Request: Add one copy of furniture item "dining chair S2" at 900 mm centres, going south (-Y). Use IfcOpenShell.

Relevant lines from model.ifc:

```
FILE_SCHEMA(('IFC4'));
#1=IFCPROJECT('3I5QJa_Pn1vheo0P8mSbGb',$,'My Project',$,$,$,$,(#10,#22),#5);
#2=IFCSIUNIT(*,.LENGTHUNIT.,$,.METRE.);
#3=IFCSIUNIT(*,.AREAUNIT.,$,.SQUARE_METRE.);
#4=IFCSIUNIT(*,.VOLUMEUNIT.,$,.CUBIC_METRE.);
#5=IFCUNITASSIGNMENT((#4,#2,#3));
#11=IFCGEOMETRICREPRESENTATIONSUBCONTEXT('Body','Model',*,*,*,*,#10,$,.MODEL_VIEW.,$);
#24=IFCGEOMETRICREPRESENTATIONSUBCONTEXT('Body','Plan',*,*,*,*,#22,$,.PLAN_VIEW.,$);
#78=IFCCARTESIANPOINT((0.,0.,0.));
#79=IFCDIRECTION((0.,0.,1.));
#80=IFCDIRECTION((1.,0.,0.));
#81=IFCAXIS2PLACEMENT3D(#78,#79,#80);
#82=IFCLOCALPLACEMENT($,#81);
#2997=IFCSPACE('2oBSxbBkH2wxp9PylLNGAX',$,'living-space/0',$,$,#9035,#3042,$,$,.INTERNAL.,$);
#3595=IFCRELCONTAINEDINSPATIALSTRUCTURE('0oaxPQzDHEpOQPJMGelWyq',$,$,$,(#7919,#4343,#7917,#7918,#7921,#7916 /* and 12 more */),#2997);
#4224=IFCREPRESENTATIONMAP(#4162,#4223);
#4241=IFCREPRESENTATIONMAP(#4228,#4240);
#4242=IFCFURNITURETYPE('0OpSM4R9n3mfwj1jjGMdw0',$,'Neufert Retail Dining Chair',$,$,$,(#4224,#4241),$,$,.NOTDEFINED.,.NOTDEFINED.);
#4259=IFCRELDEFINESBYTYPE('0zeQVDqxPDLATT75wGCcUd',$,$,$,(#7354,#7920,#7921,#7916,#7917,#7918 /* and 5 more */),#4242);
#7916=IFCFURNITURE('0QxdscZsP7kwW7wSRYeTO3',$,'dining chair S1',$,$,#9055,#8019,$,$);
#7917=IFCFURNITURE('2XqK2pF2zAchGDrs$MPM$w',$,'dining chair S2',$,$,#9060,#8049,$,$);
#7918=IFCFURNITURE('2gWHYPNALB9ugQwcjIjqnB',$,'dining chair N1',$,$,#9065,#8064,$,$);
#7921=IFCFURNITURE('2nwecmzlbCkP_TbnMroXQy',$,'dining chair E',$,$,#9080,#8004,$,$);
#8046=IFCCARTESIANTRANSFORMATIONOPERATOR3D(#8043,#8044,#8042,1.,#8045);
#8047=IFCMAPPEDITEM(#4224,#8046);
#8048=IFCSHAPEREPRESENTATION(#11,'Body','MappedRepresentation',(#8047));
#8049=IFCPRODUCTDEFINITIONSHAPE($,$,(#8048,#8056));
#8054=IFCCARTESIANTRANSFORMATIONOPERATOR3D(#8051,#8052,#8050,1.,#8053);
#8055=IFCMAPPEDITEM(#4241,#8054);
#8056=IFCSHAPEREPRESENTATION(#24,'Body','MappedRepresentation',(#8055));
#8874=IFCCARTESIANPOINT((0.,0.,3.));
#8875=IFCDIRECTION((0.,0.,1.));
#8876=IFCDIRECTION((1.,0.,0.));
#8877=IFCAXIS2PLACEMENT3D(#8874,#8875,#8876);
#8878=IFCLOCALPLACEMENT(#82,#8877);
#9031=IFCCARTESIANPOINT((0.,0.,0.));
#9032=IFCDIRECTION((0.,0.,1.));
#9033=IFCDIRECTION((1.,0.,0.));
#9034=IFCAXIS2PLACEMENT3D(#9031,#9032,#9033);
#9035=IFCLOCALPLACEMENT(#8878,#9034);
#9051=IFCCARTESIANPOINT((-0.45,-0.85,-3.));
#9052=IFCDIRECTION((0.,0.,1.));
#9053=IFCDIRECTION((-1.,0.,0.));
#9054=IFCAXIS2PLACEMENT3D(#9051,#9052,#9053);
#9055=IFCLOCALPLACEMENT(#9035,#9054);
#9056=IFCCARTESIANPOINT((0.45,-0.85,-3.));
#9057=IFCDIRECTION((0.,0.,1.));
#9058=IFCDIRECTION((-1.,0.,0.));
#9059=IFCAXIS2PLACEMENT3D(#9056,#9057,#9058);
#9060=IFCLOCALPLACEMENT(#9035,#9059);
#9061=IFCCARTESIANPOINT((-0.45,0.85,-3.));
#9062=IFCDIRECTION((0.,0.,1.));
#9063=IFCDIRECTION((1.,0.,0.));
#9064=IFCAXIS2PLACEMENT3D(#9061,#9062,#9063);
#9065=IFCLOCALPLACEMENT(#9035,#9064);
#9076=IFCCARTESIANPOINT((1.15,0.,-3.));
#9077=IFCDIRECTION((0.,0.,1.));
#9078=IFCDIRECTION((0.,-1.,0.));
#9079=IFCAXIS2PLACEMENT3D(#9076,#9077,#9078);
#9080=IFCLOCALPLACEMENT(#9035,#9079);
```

```python
import numpy as np
import ifcopenshell
import ifcopenshell.api.geometry
import ifcopenshell.api.root
import ifcopenshell.util.element
import ifcopenshell.util.placement
import ifcopenshell.util.unit

model = ifcopenshell.open("model.ifc")
unit_scale = ifcopenshell.util.unit.calculate_unit_scale(model)

source = model.by_guid("2XqK2pF2zAchGDrs$MPM$w")
base = ifcopenshell.util.placement.get_local_placement(source.ObjectPlacement)
step = np.array([0.0, -1.0, 0.0]) * 0.9 / unit_scale

for i in range(1, 2):
    copy = ifcopenshell.api.root.copy_class(model, product=source)
    copy.Representation = ifcopenshell.util.element.copy_deep(
        model, source.Representation, exclude=["IfcGeometricRepresentationContext", "IfcRepresentationMap"]
    )
    matrix = base.copy()
    matrix[:3, 3] += i * step
    print("added at", matrix[:3, 3].round(3) + 0.0)
    ifcopenshell.api.geometry.edit_object_placement(model, product=copy, matrix=matrix, is_si=False)

model.write("model_updated.ifc")
```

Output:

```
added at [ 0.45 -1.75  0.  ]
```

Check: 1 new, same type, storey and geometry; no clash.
